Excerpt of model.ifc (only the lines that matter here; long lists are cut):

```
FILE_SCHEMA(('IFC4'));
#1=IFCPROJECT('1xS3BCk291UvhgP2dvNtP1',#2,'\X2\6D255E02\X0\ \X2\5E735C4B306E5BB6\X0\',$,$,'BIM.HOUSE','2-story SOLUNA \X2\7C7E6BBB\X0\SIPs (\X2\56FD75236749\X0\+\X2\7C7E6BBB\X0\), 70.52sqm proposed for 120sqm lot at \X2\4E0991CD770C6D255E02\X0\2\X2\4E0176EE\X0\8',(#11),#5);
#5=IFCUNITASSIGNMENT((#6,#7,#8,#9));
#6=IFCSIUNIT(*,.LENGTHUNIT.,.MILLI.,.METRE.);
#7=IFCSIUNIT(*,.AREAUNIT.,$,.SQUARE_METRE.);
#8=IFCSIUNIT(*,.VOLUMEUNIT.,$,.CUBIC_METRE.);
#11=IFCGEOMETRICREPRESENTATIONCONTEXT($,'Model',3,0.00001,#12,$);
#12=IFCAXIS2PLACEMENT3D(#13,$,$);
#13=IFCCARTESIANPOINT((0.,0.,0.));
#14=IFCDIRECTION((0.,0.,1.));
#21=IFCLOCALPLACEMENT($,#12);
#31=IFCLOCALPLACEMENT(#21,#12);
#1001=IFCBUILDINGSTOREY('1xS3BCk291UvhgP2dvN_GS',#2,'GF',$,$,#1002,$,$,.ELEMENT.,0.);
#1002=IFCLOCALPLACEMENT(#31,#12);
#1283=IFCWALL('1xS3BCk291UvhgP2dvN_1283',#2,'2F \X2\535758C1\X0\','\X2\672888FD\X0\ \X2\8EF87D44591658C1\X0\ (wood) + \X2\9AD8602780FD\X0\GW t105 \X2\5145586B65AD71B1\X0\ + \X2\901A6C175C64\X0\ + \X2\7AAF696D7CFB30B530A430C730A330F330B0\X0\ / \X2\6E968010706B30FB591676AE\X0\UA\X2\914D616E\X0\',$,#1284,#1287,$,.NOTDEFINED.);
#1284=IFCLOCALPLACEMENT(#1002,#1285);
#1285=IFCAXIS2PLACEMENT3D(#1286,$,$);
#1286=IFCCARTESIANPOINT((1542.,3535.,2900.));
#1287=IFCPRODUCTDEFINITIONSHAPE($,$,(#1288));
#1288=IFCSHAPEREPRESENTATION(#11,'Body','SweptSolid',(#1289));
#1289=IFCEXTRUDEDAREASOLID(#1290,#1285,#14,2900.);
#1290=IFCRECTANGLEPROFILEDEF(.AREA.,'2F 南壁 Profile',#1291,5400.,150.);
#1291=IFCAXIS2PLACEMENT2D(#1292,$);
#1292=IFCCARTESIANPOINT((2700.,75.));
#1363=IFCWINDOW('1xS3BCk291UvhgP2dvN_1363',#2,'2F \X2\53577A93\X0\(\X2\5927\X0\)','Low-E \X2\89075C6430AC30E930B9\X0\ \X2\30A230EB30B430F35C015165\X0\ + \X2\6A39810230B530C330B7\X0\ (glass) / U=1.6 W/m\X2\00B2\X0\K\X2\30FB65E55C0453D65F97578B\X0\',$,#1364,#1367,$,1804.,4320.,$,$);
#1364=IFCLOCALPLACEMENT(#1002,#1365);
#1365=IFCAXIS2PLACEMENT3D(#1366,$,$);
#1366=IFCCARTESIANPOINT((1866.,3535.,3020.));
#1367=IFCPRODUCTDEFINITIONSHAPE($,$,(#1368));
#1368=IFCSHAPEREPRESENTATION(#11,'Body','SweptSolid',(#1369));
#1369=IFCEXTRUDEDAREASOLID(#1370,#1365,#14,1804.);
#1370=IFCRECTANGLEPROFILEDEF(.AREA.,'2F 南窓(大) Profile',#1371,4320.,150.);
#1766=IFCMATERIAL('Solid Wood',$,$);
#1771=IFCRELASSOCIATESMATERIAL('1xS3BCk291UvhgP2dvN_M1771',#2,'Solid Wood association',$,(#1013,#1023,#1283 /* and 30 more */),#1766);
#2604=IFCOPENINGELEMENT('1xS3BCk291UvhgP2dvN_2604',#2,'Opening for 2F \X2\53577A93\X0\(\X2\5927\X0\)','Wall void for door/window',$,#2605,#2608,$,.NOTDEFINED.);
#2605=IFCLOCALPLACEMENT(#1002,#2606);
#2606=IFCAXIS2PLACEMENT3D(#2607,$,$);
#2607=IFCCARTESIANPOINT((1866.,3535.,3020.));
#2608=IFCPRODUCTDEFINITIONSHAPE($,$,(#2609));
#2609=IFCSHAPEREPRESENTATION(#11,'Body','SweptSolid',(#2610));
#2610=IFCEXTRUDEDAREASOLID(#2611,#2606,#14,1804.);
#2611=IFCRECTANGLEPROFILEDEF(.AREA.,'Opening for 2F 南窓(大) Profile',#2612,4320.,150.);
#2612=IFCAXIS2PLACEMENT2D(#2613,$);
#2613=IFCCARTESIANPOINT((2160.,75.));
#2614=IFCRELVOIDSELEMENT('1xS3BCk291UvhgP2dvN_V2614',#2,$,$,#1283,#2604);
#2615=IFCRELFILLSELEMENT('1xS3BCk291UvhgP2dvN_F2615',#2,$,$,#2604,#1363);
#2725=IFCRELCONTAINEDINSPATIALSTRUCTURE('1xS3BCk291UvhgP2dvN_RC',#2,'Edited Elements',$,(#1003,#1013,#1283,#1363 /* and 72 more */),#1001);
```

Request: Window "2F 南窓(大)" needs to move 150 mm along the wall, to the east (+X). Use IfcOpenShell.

```python
import ifcopenshell
import ifcopenshell.api.geometry
import ifcopenshell.util.placement

model = ifcopenshell.open("model.ifc")

window = model.by_guid("1xS3BCk291UvhgP2dvN_1363")
opening = window.FillsVoids[0].RelatingOpeningElement
wall = opening.VoidsElements[0].RelatingBuildingElement

wall_matrix = ifcopenshell.util.placement.get_local_placement(wall.ObjectPlacement)
shift = wall_matrix[:3, 0] * 150.0
before = ifcopenshell.util.placement.get_local_placement(window.ObjectPlacement)[:3, 3].copy()

# The window is not placed relative to its opening, so move both.
for product in (opening, window):
    matrix = ifcopenshell.util.placement.get_local_placement(product.ObjectPlacement)
    matrix[:3, 3] += shift
    ifcopenshell.api.geometry.edit_object_placement(model, product=product, matrix=matrix, is_si=False)

after = ifcopenshell.util.placement.get_local_placement(window.ObjectPlacement)[:3, 3]
print("window moved by", (after - before).round(3) + 0.0)

model.write("model_updated.ifc")
```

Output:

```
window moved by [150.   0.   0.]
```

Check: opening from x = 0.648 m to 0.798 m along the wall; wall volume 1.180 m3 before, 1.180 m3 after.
